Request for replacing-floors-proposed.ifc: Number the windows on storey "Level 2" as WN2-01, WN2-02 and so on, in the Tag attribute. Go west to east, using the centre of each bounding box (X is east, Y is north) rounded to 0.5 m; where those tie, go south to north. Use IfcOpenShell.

First a look at what the model holds.

```python
import ifcopenshell
import ifcopenshell.util.element
import ifcopenshell.util.placement

model = ifcopenshell.open("replacing-floors-proposed.ifc")
print(model.schema)
storey = next(s for s in model.by_type("IfcBuildingStorey") if s.Name == "Level 2")
windows = [e for e in ifcopenshell.util.element.get_decomposition(storey) if e.is_a("IfcWindow")]
for e in sorted(windows, key=lambda e: e.id()):
    origin = ifcopenshell.util.placement.get_local_placement(e.ObjectPlacement)[:3, 3]
    print(e.id(), e.Tag, e.Name, origin.round(2) + 0.0, sep=" | ")
```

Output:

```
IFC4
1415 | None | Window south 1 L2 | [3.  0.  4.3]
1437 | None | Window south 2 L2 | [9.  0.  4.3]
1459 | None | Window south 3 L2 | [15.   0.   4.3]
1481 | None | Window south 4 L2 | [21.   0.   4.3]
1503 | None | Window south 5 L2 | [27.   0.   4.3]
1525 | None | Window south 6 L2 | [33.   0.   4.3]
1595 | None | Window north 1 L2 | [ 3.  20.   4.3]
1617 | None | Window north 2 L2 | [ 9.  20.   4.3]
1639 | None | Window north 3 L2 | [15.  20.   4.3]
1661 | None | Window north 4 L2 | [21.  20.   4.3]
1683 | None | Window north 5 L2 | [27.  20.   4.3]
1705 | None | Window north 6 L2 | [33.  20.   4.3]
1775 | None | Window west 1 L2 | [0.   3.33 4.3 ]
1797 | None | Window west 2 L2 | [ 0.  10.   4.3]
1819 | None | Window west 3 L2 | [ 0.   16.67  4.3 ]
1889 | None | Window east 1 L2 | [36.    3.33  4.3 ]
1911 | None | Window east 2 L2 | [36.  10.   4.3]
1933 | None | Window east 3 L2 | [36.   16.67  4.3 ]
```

```python
import ifcopenshell
import ifcopenshell.geom
import ifcopenshell.util.element
import ifcopenshell.util.shape

model = ifcopenshell.open("replacing-floors-proposed.ifc")
settings = ifcopenshell.geom.settings()
settings.set("use-world-coords", True)


def centre(element):
    shape = ifcopenshell.geom.create_shape(settings, element)
    return ifcopenshell.util.shape.get_bbox_centroid(shape.geometry)


storey = next(s for s in model.by_type("IfcBuildingStorey") if s.Name == "Level 2")
windows = [e for e in ifcopenshell.util.element.get_decomposition(storey) if e.is_a("IfcWindow")]

# Insertion points can sit at a corner or the storey origin, so sort by the geometry (in metres).
centres = {e: centre(e) for e in windows}
windows.sort(key=lambda e: (round(centres[e][0] / 0.5), centres[e][1]))

for i, e in enumerate(windows, start=1):
    number = f"WN2-{i:02d}"
    e.Tag = number
    print(e.id(), number)

model.write("replacing-floors-proposed_updated.ifc")
```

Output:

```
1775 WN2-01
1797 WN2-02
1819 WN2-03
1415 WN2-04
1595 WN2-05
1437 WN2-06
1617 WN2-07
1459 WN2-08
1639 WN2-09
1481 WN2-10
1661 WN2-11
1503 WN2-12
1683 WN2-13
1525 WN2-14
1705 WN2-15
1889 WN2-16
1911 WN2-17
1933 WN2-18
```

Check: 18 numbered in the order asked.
